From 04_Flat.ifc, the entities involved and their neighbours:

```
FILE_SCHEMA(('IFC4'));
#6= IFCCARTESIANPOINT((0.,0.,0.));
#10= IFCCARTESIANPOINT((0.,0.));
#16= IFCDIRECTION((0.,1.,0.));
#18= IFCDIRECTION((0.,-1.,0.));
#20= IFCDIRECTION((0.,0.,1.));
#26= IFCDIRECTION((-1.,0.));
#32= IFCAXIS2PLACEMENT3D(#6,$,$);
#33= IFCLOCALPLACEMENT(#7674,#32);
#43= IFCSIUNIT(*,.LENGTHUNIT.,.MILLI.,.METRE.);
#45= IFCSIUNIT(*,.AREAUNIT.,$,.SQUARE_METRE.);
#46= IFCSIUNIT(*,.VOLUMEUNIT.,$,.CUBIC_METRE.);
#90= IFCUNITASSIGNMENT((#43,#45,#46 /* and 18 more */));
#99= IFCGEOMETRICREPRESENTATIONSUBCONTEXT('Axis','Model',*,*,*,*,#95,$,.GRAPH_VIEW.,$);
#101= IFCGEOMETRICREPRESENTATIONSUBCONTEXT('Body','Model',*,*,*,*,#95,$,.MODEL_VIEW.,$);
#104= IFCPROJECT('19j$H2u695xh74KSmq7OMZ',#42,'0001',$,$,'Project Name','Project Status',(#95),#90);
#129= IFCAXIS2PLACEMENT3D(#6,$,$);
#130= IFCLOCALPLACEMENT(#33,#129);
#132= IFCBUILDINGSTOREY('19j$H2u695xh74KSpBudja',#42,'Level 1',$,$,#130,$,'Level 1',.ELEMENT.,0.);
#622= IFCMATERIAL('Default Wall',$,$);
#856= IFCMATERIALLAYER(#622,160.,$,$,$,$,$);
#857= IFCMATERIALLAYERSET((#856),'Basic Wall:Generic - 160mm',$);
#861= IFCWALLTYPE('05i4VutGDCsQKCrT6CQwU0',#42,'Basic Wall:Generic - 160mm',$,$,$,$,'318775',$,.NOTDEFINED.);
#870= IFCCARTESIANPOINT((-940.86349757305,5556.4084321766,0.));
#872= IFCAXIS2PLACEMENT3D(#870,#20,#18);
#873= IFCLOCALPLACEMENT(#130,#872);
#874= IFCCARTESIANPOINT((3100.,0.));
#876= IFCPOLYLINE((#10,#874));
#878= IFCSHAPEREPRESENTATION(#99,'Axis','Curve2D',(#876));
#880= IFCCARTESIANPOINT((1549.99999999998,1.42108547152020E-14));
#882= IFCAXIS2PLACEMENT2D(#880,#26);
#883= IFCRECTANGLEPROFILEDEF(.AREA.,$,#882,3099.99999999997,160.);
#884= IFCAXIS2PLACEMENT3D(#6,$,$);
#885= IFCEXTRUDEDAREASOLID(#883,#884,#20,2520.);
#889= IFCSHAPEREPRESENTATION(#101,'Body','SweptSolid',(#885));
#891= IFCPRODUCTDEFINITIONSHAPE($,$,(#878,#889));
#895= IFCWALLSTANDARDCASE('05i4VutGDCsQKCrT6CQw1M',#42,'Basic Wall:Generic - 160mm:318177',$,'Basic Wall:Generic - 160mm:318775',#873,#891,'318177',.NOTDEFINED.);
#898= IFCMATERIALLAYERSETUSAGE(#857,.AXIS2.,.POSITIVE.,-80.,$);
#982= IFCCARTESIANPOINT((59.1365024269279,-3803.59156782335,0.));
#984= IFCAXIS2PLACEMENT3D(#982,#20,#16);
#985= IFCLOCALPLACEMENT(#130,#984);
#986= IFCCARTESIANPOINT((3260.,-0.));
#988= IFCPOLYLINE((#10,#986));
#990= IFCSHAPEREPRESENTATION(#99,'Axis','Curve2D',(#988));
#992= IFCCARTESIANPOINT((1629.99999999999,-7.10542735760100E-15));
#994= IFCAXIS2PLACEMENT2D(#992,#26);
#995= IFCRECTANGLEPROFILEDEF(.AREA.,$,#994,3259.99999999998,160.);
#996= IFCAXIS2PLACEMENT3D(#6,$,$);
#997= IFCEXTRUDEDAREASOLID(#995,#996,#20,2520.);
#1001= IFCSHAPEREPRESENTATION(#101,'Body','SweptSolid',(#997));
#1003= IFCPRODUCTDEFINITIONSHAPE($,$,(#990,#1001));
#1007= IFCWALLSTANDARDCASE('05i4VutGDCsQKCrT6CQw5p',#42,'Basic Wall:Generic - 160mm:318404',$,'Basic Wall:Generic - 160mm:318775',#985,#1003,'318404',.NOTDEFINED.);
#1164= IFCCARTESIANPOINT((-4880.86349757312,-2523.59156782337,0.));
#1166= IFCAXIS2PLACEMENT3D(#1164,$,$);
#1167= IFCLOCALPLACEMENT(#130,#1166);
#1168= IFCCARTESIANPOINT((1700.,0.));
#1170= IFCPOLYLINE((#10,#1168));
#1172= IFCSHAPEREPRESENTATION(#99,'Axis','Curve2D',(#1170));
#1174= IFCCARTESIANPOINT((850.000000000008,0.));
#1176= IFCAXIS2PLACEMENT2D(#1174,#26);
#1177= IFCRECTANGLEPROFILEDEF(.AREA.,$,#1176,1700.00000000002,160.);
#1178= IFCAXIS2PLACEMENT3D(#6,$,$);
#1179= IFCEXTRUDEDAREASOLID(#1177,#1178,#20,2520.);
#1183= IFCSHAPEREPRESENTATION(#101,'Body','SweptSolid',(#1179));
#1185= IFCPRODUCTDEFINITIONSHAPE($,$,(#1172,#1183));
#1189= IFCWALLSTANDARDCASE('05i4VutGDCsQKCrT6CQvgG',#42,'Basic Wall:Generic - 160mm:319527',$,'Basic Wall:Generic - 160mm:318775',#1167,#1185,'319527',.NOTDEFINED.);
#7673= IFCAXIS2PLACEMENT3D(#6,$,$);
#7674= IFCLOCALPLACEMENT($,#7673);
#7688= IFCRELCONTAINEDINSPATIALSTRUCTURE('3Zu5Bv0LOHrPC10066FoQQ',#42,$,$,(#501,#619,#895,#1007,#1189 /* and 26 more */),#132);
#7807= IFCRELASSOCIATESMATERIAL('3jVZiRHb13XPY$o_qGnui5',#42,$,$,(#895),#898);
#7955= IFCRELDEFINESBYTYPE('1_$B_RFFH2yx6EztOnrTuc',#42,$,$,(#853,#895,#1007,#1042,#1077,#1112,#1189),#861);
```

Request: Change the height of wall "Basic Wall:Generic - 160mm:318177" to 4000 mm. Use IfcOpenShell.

```python
import ifcopenshell
import ifcopenshell.geom
import ifcopenshell.util.representation
import ifcopenshell.util.shape

model = ifcopenshell.open("04_Flat.ifc")
settings = ifcopenshell.geom.settings()


def volume(element):
    """Net volume in cubic metres, openings subtracted."""
    shape = ifcopenshell.geom.create_shape(settings, element)
    return ifcopenshell.util.shape.get_volume(shape.geometry)


wall = model.by_guid("05i4VutGDCsQKCrT6CQw1M")
before = volume(wall)

body = ifcopenshell.util.representation.get_representation(wall, "Model", "Body")
solid = body.Items[0]
old_height = solid.Depth
solid.Depth = 4000.0
after = volume(wall)

print(f"height {old_height:g} -> {solid.Depth:g}, volume {before:.3f} -> {after:.3f} m3")

model.write("04_Flat_rev.ifc")
```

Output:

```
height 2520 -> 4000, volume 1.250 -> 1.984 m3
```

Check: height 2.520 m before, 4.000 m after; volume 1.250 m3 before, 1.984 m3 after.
